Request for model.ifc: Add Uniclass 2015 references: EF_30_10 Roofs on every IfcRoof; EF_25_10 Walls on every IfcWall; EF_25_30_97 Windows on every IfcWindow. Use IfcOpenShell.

First a look at what the model holds.

```python
import ifcopenshell

model = ifcopenshell.open("model.ifc")
print(model.schema)
print("classifications:", [c.Name for c in model.by_type("IfcClassification")])
for ifc_class in ("IfcDoor", "IfcRoof", "IfcStair", "IfcWall", "IfcWindow"):
    print(ifc_class, len(model.by_type(ifc_class)))
```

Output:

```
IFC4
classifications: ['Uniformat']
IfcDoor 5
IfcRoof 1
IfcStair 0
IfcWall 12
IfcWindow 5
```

```python
import ifcopenshell
import ifcopenshell.api.classification

model = ifcopenshell.open("model.ifc")

system = ifcopenshell.api.classification.add_classification(model, classification="Uniclass 2015")

codes = {
    "IfcRoof": ("EF_30_10", "Roofs"),
    "IfcWall": ("EF_25_10", "Walls"),
    "IfcWindow": ("EF_25_30_97", "Windows"),
}
for ifc_class, (code, name) in codes.items():
    products = model.by_type(ifc_class)
    ifcopenshell.api.classification.add_reference(
        model, products=products, classification=system, identification=code, name=name
    )
    print(code, len(products))

model.write("model_edited.ifc")
```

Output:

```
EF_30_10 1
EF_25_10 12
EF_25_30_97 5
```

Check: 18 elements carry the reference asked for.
